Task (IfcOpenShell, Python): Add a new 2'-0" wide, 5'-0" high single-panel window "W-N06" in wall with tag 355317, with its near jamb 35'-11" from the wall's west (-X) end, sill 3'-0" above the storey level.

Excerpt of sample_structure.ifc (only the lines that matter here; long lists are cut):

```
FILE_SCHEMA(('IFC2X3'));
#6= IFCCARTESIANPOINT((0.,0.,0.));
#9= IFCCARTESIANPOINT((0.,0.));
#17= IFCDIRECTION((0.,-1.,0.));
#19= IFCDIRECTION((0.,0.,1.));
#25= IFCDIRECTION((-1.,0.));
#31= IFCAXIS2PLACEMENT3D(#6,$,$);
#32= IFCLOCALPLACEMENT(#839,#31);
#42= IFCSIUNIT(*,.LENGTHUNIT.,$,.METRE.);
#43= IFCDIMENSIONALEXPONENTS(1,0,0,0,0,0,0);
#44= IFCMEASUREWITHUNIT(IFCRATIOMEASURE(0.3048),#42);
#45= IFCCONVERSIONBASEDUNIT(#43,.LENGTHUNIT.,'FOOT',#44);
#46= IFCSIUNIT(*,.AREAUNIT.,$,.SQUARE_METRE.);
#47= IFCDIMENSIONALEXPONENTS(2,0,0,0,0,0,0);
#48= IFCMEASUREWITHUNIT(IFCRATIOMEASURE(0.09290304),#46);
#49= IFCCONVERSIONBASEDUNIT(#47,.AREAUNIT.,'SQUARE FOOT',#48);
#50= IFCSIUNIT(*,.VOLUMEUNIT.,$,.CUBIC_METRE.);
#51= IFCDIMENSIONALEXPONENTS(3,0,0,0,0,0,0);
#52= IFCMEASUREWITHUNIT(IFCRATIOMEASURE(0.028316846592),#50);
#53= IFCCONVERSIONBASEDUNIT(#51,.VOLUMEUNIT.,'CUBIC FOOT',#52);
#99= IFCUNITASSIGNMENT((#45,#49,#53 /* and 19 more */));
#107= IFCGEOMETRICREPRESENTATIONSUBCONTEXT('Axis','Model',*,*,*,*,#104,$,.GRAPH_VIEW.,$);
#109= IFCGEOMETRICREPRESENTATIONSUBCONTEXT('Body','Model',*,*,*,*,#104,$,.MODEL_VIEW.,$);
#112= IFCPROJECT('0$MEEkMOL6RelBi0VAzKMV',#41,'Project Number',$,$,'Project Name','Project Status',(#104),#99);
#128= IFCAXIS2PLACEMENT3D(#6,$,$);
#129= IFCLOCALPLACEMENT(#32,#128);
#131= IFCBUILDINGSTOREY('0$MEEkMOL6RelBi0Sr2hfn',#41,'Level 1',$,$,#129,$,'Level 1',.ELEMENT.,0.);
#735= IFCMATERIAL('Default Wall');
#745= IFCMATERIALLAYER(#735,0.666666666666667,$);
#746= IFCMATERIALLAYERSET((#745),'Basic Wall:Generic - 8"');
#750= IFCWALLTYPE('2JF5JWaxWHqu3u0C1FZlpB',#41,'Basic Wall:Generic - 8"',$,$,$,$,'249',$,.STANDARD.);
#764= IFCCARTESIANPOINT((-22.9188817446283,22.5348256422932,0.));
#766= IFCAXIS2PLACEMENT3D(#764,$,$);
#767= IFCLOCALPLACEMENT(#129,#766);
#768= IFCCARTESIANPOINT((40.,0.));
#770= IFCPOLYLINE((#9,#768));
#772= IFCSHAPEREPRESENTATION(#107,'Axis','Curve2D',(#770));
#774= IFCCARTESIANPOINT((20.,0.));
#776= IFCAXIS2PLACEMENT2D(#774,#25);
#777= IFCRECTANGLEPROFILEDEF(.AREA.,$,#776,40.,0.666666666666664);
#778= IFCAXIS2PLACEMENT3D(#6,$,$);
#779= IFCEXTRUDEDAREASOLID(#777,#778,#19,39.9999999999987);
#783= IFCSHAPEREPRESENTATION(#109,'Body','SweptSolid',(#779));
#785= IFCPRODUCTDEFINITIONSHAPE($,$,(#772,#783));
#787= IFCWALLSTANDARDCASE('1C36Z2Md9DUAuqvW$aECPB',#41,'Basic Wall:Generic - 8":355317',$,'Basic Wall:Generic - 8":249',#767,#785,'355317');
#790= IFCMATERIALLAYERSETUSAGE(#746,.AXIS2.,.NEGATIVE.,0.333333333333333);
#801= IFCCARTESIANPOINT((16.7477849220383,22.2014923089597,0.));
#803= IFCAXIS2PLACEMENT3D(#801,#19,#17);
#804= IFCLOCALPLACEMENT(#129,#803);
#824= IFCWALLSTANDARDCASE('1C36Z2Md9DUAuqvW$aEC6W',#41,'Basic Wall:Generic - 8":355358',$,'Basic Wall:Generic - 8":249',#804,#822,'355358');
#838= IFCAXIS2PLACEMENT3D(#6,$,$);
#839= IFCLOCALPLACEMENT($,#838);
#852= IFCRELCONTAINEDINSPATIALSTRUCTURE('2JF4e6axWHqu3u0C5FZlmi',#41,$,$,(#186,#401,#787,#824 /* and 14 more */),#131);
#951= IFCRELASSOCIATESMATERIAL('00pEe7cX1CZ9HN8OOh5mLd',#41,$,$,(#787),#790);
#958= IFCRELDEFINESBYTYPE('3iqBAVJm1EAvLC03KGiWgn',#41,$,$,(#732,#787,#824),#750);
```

```python
import numpy as np
import ifcopenshell
import ifcopenshell.api.feature
import ifcopenshell.api.geometry
import ifcopenshell.api.root
import ifcopenshell.api.spatial
import ifcopenshell.api.type
import ifcopenshell.geom
import ifcopenshell.util.element
import ifcopenshell.util.placement
import ifcopenshell.util.representation
import ifcopenshell.util.shape
import ifcopenshell.util.unit

model = ifcopenshell.open("sample_structure.ifc")
unit_scale = ifcopenshell.util.unit.calculate_unit_scale(model)
settings = ifcopenshell.geom.settings()


def volume(element):
    """Net volume in cubic metres, openings subtracted."""
    shape = ifcopenshell.geom.create_shape(settings, element)
    return ifcopenshell.util.shape.get_volume(shape.geometry)


wall = model.by_id(787)
storey = ifcopenshell.util.element.get_container(wall, ifc_class="IfcBuildingStorey")
context = ifcopenshell.util.representation.get_context(model, "Model", "Body", "MODEL_VIEW")
before = volume(wall)

width, height, from_end, sill = 0.6096, 1.524, 10.9474, 0.9144  # metres

# The wall runs along its own X axis, and the end named is its -X end.
wall_shape = ifcopenshell.geom.create_shape(settings, wall)
x, y, z = ifcopenshell.util.shape.get_vertices(wall_shape.geometry).T
start = x.min() + from_end
face, thickness = float(y.min()), float(y.max() - y.min())
wall_matrix = ifcopenshell.util.placement.get_local_placement(wall.ObjectPlacement)
level = ifcopenshell.util.placement.get_local_placement(storey.ObjectPlacement)[2, 3]


def in_wall(x, y):
    """Placement at x, y metres in the wall's axes, at sill height."""
    matrix = wall_matrix.copy()
    matrix[:, 3] = wall_matrix @ np.array([x / unit_scale, y / unit_scale, 0.0, 1.0])
    matrix[2, 3] = level + sill / unit_scale
    return matrix


# Opening: a box that overshoots both wall faces by 50 mm.
opening = ifcopenshell.api.root.create_entity(model, ifc_class="IfcOpeningElement")
box = ifcopenshell.api.geometry.add_wall_representation(
    model, context=context, length=width, height=height, thickness=thickness + 0.1
)
ifcopenshell.api.geometry.assign_representation(model, product=opening, representation=box)
ifcopenshell.api.geometry.edit_object_placement(model, product=opening, matrix=in_wall(start, face - 0.05), is_si=False)
ifcopenshell.api.feature.add_feature(model, feature=opening, element=wall)

window = ifcopenshell.api.root.create_entity(model, ifc_class="IfcWindow", name="W-N06")
window.OverallWidth, window.OverallHeight = width / unit_scale, height / unit_scale
body = ifcopenshell.api.geometry.add_window_representation(
    model,
    context=context,
    overall_width=window.OverallWidth,
    overall_height=window.OverallHeight,
    partition_type="SINGLE_PANEL",
)
ifcopenshell.api.geometry.assign_representation(model, product=window, representation=body)
ifcopenshell.api.spatial.assign_container(model, products=[window], relating_structure=storey)
fills = ifcopenshell.api.feature.add_filling(model, opening=opening, element=window)
fills.OwnerHistory = window.OwnerHistory  # required in IFC2X3

# IFC2X3 keeps the operation on the window style.
style = ifcopenshell.api.root.create_entity(model, ifc_class="IfcWindowStyle", name="W-N06")
style.OperationType, style.ConstructionType = "SINGLE_PANEL", "NOTDEFINED"
style.ParameterTakesPrecedence = style.Sizeable = False
ifcopenshell.api.type.assign_type(model, related_objects=[window], relating_type=style)

# Centre the window in the wall's thickness.
ifcopenshell.api.geometry.edit_object_placement(model, product=window, matrix=in_wall(start, face), is_si=False)
window_shape = ifcopenshell.geom.create_shape(settings, window)
depth = ifcopenshell.util.shape.get_vertices(window_shape.geometry)[:, 1]
offset = face + thickness / 2 - (depth.min() + depth.max()) / 2
ifcopenshell.api.geometry.edit_object_placement(model, product=window, matrix=in_wall(start, offset), is_si=False)

after = volume(wall)

print(f"wall volume {before:.3f} -> {after:.3f} m3")

model.write("sample_structure_v2.ifc")
```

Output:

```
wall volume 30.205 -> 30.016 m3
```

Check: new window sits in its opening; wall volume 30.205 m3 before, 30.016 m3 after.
